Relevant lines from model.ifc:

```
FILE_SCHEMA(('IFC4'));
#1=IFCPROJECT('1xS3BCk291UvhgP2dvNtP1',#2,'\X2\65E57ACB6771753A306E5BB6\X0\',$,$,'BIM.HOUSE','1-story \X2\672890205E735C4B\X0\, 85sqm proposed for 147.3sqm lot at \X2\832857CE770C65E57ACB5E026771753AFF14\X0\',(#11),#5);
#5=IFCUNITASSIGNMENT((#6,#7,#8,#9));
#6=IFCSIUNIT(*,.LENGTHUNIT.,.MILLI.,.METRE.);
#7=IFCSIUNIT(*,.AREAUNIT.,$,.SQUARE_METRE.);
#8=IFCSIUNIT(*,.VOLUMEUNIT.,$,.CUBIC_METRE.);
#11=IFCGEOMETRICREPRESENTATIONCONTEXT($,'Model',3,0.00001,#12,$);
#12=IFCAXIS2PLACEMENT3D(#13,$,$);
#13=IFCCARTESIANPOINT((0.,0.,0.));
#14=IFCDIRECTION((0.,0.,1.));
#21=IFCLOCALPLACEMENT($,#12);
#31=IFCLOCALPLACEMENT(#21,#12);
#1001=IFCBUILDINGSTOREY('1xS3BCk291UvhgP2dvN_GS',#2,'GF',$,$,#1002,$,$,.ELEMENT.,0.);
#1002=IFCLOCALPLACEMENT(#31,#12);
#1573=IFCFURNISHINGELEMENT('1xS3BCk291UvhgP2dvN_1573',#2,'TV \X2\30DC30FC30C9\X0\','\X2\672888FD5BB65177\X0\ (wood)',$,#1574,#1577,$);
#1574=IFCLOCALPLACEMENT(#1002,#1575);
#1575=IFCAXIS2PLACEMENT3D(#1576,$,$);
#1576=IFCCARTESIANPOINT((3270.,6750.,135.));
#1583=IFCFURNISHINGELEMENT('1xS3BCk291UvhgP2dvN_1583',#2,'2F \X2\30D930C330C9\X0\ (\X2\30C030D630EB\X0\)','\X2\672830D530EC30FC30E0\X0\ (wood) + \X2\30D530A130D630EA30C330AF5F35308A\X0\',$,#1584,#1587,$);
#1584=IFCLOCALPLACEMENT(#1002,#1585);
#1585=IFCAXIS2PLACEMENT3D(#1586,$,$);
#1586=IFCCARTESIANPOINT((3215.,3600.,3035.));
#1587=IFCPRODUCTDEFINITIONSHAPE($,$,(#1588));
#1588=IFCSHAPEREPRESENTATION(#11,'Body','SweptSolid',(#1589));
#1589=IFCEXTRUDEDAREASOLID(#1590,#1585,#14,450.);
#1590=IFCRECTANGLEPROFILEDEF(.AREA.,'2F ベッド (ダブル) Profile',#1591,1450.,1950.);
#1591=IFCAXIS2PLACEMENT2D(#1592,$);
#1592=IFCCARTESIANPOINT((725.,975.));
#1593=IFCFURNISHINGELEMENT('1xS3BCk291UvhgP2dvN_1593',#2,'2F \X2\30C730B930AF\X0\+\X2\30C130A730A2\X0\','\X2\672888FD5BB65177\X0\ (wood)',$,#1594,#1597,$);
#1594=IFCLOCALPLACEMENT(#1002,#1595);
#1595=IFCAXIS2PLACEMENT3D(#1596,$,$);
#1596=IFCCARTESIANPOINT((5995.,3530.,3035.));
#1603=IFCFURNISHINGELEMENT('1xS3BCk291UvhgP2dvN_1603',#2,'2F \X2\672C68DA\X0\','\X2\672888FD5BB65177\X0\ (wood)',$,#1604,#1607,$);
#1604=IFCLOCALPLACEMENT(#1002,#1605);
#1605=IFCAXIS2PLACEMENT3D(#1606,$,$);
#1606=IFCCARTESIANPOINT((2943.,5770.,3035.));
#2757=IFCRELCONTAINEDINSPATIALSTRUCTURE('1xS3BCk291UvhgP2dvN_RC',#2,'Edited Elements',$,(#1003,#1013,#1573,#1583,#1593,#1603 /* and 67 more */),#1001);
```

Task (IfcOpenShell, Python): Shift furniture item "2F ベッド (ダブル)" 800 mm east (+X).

```python
import ifcopenshell
import ifcopenshell.api.geometry
import ifcopenshell.util.placement
import ifcopenshell.util.unit

model = ifcopenshell.open("model.ifc")
unit_scale = ifcopenshell.util.unit.calculate_unit_scale(model)

item = model.by_guid("1xS3BCk291UvhgP2dvN_1583")
matrix = ifcopenshell.util.placement.get_local_placement(item.ObjectPlacement)
matrix[0, 3] += 0.8 / unit_scale
ifcopenshell.api.geometry.edit_object_placement(model, product=item, matrix=matrix, is_si=False)

print(ifcopenshell.util.placement.get_local_placement(item.ObjectPlacement).round(3) + 0.0)

model.write("model_v2.ifc")
```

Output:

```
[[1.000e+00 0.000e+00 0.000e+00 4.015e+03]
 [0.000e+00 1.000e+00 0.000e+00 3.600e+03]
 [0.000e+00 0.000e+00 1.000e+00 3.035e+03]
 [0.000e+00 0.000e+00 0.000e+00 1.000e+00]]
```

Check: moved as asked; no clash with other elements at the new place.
